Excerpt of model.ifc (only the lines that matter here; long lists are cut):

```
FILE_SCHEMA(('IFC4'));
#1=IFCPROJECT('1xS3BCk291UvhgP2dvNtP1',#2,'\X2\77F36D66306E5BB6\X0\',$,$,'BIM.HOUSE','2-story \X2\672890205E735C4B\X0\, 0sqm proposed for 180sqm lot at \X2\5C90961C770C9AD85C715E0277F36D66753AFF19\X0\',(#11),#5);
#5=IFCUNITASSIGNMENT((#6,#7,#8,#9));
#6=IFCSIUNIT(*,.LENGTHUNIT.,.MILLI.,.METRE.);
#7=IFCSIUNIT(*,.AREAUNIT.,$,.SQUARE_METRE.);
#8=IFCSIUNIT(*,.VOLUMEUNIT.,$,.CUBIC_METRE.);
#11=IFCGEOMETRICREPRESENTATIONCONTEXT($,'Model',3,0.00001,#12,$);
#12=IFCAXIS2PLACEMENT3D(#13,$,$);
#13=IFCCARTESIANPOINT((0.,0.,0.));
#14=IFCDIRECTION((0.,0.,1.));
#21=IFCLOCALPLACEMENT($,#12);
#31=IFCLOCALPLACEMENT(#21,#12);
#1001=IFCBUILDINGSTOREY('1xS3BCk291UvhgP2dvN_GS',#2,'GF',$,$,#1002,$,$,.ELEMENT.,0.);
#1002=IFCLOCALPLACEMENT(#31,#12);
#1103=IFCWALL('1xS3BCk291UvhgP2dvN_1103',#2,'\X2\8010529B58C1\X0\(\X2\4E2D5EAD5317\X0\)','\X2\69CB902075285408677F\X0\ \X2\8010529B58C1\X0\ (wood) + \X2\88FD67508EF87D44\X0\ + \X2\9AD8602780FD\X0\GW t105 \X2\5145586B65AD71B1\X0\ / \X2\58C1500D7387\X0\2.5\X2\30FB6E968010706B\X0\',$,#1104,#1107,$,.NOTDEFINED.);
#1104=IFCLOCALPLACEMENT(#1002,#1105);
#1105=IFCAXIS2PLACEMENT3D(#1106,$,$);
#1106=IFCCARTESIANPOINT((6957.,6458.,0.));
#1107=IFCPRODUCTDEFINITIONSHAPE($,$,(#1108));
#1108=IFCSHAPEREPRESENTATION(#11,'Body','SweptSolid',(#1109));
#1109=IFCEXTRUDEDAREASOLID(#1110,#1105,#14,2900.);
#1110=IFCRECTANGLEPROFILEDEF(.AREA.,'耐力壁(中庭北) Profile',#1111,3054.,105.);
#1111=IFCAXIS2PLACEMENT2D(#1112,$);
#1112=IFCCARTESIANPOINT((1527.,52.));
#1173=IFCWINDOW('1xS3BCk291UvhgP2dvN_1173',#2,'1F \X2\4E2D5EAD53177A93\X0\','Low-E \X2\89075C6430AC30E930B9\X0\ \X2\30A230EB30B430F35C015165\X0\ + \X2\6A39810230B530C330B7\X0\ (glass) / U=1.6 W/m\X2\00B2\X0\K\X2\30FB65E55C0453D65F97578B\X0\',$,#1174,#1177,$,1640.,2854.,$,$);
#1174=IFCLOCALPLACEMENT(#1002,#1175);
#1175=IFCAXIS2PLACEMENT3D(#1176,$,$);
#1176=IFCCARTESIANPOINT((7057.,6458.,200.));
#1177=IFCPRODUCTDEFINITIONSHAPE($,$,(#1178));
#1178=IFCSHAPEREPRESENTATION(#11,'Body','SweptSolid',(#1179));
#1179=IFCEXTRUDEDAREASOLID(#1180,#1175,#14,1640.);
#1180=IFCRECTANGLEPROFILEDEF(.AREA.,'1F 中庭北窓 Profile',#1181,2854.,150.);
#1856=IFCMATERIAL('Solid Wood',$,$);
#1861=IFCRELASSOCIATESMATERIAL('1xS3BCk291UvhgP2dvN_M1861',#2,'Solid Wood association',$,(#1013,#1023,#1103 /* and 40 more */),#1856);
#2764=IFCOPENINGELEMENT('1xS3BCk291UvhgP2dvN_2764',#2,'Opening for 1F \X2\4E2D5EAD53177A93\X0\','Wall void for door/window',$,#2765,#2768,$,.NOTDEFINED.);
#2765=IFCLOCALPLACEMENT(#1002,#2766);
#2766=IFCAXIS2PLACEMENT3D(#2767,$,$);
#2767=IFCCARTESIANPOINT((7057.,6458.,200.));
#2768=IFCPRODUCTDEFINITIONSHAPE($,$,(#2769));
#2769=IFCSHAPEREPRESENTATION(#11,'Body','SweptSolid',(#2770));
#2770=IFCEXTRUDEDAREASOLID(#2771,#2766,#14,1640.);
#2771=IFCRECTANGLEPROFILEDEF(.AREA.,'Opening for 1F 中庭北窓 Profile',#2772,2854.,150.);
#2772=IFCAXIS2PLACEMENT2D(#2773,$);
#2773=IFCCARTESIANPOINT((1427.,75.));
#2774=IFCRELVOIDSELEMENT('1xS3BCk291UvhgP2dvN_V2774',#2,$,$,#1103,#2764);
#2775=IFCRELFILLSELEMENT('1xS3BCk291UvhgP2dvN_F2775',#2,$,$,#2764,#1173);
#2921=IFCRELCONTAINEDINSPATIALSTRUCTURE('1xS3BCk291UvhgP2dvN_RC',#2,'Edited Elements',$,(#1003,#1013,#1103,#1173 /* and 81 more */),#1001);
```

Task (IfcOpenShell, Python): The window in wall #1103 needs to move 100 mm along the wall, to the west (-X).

```python
import ifcopenshell
import ifcopenshell.api.geometry
import ifcopenshell.util.placement

model = ifcopenshell.open("model.ifc")

window = model.by_guid("1xS3BCk291UvhgP2dvN_1173")
opening = window.FillsVoids[0].RelatingOpeningElement
wall = opening.VoidsElements[0].RelatingBuildingElement

wall_matrix = ifcopenshell.util.placement.get_local_placement(wall.ObjectPlacement)
shift = wall_matrix[:3, 0] * -100.0
before = ifcopenshell.util.placement.get_local_placement(window.ObjectPlacement)[:3, 3].copy()

# The window is not placed relative to its opening, so move both.
for product in (opening, window):
    matrix = ifcopenshell.util.placement.get_local_placement(product.ObjectPlacement)
    matrix[:3, 3] += shift
    ifcopenshell.api.geometry.edit_object_placement(model, product=product, matrix=matrix, is_si=False)

after = ifcopenshell.util.placement.get_local_placement(window.ObjectPlacement)[:3, 3]
print("window moved by", (after - before).round(3) + 0.0)

model.write("model_edited.ifc")
```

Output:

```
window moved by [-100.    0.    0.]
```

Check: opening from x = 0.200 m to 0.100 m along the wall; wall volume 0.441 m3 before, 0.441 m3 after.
